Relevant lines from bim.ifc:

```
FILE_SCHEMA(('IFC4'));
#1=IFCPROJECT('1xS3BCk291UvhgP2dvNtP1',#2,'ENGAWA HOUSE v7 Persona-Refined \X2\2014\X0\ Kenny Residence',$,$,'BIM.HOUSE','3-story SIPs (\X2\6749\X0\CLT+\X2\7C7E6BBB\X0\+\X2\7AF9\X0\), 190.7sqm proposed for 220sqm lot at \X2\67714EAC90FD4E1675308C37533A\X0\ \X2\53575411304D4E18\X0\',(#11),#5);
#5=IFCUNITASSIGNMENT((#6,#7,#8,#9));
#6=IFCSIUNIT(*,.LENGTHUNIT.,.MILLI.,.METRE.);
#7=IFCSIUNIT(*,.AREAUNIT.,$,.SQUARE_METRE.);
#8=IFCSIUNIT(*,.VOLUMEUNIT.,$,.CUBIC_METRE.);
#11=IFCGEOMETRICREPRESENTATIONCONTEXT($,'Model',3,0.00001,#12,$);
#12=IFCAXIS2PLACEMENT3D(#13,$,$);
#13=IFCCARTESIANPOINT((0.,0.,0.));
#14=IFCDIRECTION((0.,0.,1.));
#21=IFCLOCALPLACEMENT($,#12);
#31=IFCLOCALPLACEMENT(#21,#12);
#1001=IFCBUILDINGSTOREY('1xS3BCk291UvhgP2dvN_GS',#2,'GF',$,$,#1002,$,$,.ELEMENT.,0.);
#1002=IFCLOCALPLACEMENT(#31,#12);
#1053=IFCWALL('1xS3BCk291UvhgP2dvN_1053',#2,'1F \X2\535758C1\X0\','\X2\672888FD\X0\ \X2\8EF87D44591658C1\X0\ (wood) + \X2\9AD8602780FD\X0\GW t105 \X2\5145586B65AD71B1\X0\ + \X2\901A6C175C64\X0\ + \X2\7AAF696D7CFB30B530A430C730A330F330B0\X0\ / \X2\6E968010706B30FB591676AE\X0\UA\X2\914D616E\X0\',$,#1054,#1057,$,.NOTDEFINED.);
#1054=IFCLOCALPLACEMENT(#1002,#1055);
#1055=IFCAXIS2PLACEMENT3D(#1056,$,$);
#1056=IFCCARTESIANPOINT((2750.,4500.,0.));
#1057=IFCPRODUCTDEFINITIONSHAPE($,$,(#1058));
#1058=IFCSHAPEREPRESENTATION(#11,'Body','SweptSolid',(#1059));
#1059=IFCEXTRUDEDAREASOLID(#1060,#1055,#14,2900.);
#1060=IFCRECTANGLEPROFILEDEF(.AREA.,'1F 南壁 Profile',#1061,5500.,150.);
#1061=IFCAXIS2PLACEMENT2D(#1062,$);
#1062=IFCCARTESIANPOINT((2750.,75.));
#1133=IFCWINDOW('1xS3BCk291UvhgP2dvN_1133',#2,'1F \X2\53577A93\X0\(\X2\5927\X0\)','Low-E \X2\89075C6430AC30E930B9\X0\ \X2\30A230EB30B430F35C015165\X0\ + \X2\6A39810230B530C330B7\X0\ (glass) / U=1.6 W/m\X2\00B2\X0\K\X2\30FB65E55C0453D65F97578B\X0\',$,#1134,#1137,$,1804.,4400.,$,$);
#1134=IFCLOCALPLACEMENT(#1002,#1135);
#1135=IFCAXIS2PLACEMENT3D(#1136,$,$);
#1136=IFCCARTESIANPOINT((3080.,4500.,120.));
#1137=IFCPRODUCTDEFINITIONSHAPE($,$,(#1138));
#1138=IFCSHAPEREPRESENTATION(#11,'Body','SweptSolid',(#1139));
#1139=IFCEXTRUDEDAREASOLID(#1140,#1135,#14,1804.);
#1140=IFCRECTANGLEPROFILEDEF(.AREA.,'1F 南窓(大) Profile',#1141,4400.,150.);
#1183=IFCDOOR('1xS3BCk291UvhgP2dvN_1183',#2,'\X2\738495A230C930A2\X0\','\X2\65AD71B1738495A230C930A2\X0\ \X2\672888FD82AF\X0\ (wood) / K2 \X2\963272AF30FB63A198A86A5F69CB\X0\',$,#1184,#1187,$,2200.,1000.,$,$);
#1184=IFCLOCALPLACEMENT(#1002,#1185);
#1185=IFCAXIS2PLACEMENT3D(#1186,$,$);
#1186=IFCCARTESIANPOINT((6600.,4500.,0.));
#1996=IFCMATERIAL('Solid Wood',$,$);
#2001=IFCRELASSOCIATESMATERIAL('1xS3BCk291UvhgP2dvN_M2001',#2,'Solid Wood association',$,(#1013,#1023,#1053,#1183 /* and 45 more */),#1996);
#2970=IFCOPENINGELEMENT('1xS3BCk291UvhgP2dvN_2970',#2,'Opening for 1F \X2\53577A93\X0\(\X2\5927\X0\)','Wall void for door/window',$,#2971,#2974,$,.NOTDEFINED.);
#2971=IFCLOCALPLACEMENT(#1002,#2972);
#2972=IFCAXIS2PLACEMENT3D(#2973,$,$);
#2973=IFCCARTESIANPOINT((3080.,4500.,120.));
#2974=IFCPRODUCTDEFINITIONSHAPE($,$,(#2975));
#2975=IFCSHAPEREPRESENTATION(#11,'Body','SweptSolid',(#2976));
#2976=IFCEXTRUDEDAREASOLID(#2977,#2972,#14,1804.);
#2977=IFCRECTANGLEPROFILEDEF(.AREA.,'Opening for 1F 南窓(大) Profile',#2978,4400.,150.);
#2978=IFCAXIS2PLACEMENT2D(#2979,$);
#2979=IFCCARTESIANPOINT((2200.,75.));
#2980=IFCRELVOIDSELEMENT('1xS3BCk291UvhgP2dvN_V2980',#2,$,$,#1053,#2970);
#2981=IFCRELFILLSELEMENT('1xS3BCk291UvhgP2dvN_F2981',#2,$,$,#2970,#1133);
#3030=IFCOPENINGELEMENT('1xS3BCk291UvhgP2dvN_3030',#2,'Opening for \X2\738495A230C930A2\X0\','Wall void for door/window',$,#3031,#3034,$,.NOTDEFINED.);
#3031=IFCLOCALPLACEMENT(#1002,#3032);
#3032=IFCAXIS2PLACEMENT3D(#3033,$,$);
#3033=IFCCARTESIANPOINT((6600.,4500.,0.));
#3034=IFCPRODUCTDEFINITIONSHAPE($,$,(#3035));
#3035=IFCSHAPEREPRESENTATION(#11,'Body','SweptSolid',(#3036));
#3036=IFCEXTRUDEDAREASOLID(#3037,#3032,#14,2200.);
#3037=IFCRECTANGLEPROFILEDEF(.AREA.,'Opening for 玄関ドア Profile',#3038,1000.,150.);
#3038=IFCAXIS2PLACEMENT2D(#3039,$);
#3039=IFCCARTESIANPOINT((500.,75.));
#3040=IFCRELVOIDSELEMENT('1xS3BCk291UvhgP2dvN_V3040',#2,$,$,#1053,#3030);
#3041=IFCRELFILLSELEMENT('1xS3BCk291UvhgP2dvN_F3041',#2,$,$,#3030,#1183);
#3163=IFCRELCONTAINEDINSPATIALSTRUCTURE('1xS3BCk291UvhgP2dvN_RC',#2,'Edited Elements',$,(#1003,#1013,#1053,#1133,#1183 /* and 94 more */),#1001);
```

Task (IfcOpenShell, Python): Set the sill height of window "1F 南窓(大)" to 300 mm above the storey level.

```python
import numpy as np
import ifcopenshell
import ifcopenshell.api.geometry
import ifcopenshell.geom
import ifcopenshell.util.element
import ifcopenshell.util.placement
import ifcopenshell.util.shape
import ifcopenshell.util.unit

model = ifcopenshell.open("bim.ifc")
unit_scale = ifcopenshell.util.unit.calculate_unit_scale(model)

window = model.by_guid("1xS3BCk291UvhgP2dvN_1133")
opening = window.FillsVoids[0].RelatingOpeningElement
storey = ifcopenshell.util.element.get_container(window, ifc_class="IfcBuildingStorey")
level = ifcopenshell.util.placement.get_local_placement(storey.ObjectPlacement)[2, 3]

# The opening's origin need not be at the sill, so measure its lowest point.
shape = ifcopenshell.geom.create_shape(ifcopenshell.geom.settings(), opening)
bottom = ifcopenshell.util.shape.get_shape_bottom_elevation(shape, shape.geometry) / unit_scale
dz = level + 0.3 / unit_scale - bottom

shift = np.array([0.0, 0.0, dz])
# The window is not placed relative to its opening, so move both.
for product in (opening, window):
    matrix = ifcopenshell.util.placement.get_local_placement(product.ObjectPlacement)
    matrix[:3, 3] += shift
    ifcopenshell.api.geometry.edit_object_placement(model, product=product, matrix=matrix, is_si=False)

print(f"moved by {dz * unit_scale:+.3f} m")

model.write("bim_edited.ifc")
```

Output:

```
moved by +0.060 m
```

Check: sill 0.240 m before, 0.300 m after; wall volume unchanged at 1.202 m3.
